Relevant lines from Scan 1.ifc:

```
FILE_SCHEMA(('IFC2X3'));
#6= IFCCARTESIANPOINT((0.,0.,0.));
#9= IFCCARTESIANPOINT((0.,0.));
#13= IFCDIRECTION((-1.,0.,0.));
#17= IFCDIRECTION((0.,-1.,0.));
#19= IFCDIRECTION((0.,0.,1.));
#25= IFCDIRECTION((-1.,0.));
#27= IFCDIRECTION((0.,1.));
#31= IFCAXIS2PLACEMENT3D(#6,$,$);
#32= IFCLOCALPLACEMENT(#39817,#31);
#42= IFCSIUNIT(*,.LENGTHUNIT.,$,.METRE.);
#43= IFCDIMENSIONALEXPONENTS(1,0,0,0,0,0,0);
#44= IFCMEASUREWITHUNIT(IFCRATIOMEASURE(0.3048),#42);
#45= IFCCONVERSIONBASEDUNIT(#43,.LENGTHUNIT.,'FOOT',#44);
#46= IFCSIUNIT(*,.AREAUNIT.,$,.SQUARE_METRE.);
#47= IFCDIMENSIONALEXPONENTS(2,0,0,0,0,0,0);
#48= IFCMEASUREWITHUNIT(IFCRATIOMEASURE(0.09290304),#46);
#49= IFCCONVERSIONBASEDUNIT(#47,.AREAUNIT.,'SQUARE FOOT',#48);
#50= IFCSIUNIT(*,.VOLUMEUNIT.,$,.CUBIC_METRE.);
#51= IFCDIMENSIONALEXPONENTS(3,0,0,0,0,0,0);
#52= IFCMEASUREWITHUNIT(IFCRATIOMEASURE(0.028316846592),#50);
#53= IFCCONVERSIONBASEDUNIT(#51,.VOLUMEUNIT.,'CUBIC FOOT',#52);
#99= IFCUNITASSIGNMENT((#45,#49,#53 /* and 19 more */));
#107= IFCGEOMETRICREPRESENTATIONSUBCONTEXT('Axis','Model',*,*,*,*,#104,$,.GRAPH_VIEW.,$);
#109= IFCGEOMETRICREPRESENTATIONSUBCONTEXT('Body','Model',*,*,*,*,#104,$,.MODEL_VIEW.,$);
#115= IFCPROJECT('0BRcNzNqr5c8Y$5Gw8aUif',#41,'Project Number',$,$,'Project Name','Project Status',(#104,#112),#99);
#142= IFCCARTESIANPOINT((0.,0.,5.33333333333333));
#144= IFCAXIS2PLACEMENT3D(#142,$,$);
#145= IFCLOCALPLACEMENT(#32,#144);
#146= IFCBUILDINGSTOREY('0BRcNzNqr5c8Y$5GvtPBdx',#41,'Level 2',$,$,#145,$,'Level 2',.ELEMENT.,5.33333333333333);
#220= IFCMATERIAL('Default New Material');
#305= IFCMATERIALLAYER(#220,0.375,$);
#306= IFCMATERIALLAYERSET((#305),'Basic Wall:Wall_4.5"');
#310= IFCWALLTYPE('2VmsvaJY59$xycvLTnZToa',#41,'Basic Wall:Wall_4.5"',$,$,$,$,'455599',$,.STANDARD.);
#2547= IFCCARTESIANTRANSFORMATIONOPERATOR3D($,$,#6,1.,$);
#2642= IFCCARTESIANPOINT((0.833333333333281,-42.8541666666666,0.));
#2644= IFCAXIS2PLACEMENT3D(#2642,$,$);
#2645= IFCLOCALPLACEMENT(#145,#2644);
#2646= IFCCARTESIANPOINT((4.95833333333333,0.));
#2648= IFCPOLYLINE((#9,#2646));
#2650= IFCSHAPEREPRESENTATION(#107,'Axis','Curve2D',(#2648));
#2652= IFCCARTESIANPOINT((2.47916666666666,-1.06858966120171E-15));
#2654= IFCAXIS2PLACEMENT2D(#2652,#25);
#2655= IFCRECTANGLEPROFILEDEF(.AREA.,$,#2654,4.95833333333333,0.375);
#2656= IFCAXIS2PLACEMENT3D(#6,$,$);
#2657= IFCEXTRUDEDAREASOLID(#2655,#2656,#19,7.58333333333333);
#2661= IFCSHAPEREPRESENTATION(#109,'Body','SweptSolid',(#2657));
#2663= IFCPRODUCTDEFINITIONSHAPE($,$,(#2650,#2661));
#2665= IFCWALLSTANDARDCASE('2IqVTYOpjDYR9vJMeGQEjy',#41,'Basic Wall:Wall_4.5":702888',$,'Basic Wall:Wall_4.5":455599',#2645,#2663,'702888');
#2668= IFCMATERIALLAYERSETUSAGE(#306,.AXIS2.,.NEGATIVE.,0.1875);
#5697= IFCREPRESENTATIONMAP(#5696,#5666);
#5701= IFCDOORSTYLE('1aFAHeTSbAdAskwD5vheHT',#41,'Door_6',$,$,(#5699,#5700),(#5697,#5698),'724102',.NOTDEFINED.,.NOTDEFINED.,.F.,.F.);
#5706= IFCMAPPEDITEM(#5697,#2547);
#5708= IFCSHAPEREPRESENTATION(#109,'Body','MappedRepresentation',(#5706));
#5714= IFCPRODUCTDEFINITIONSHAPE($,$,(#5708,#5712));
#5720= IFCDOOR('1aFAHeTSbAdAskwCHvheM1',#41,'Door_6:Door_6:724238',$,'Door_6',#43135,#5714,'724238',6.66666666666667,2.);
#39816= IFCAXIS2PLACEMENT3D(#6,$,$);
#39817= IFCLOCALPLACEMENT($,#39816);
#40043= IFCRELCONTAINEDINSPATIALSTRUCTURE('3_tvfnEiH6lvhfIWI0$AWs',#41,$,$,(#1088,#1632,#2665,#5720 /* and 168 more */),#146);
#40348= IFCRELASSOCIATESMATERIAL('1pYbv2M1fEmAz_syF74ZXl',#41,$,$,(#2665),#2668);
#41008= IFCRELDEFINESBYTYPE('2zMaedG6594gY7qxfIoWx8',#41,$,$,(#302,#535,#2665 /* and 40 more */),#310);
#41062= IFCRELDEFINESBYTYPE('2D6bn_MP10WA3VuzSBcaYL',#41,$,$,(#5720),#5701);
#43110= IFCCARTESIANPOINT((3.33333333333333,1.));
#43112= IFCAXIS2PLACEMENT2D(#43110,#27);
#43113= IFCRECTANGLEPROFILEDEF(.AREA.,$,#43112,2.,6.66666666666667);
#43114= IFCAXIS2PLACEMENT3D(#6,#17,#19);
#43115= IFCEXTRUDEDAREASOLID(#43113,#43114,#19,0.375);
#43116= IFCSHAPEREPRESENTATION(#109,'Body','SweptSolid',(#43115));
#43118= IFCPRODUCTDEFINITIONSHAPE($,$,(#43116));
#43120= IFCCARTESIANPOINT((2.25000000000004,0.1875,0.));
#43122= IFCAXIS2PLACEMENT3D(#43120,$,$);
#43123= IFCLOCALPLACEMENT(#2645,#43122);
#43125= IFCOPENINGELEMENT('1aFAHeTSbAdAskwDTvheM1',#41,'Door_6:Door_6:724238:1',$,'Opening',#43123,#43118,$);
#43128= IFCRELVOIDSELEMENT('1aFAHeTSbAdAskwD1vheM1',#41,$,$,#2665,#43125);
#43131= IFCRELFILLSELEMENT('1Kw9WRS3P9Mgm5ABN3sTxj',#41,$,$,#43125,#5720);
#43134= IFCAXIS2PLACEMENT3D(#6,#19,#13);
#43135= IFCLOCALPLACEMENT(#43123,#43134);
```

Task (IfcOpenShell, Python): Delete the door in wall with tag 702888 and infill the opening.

```python
import ifcopenshell
import ifcopenshell.api.feature
import ifcopenshell.api.root
import ifcopenshell.geom
import ifcopenshell.util.shape

model = ifcopenshell.open("Scan 1.ifc")
settings = ifcopenshell.geom.settings()


def volume(element):
    """Net volume in cubic metres, openings subtracted."""
    shape = ifcopenshell.geom.create_shape(settings, element)
    return ifcopenshell.util.shape.get_volume(shape.geometry)


door = model.by_guid("1aFAHeTSbAdAskwCHvheM1")
opening = door.FillsVoids[0].RelatingOpeningElement
wall = opening.VoidsElements[0].RelatingBuildingElement
before = volume(wall)

ifcopenshell.api.root.remove_product(model, product=door)
ifcopenshell.api.feature.remove_feature(model, feature=opening)

after = volume(wall)

print(f"wall volume {before:.3f} -> {after:.3f} m3")

model.write("Scan 1-out.ifc")
```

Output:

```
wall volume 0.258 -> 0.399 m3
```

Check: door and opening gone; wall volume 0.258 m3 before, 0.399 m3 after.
